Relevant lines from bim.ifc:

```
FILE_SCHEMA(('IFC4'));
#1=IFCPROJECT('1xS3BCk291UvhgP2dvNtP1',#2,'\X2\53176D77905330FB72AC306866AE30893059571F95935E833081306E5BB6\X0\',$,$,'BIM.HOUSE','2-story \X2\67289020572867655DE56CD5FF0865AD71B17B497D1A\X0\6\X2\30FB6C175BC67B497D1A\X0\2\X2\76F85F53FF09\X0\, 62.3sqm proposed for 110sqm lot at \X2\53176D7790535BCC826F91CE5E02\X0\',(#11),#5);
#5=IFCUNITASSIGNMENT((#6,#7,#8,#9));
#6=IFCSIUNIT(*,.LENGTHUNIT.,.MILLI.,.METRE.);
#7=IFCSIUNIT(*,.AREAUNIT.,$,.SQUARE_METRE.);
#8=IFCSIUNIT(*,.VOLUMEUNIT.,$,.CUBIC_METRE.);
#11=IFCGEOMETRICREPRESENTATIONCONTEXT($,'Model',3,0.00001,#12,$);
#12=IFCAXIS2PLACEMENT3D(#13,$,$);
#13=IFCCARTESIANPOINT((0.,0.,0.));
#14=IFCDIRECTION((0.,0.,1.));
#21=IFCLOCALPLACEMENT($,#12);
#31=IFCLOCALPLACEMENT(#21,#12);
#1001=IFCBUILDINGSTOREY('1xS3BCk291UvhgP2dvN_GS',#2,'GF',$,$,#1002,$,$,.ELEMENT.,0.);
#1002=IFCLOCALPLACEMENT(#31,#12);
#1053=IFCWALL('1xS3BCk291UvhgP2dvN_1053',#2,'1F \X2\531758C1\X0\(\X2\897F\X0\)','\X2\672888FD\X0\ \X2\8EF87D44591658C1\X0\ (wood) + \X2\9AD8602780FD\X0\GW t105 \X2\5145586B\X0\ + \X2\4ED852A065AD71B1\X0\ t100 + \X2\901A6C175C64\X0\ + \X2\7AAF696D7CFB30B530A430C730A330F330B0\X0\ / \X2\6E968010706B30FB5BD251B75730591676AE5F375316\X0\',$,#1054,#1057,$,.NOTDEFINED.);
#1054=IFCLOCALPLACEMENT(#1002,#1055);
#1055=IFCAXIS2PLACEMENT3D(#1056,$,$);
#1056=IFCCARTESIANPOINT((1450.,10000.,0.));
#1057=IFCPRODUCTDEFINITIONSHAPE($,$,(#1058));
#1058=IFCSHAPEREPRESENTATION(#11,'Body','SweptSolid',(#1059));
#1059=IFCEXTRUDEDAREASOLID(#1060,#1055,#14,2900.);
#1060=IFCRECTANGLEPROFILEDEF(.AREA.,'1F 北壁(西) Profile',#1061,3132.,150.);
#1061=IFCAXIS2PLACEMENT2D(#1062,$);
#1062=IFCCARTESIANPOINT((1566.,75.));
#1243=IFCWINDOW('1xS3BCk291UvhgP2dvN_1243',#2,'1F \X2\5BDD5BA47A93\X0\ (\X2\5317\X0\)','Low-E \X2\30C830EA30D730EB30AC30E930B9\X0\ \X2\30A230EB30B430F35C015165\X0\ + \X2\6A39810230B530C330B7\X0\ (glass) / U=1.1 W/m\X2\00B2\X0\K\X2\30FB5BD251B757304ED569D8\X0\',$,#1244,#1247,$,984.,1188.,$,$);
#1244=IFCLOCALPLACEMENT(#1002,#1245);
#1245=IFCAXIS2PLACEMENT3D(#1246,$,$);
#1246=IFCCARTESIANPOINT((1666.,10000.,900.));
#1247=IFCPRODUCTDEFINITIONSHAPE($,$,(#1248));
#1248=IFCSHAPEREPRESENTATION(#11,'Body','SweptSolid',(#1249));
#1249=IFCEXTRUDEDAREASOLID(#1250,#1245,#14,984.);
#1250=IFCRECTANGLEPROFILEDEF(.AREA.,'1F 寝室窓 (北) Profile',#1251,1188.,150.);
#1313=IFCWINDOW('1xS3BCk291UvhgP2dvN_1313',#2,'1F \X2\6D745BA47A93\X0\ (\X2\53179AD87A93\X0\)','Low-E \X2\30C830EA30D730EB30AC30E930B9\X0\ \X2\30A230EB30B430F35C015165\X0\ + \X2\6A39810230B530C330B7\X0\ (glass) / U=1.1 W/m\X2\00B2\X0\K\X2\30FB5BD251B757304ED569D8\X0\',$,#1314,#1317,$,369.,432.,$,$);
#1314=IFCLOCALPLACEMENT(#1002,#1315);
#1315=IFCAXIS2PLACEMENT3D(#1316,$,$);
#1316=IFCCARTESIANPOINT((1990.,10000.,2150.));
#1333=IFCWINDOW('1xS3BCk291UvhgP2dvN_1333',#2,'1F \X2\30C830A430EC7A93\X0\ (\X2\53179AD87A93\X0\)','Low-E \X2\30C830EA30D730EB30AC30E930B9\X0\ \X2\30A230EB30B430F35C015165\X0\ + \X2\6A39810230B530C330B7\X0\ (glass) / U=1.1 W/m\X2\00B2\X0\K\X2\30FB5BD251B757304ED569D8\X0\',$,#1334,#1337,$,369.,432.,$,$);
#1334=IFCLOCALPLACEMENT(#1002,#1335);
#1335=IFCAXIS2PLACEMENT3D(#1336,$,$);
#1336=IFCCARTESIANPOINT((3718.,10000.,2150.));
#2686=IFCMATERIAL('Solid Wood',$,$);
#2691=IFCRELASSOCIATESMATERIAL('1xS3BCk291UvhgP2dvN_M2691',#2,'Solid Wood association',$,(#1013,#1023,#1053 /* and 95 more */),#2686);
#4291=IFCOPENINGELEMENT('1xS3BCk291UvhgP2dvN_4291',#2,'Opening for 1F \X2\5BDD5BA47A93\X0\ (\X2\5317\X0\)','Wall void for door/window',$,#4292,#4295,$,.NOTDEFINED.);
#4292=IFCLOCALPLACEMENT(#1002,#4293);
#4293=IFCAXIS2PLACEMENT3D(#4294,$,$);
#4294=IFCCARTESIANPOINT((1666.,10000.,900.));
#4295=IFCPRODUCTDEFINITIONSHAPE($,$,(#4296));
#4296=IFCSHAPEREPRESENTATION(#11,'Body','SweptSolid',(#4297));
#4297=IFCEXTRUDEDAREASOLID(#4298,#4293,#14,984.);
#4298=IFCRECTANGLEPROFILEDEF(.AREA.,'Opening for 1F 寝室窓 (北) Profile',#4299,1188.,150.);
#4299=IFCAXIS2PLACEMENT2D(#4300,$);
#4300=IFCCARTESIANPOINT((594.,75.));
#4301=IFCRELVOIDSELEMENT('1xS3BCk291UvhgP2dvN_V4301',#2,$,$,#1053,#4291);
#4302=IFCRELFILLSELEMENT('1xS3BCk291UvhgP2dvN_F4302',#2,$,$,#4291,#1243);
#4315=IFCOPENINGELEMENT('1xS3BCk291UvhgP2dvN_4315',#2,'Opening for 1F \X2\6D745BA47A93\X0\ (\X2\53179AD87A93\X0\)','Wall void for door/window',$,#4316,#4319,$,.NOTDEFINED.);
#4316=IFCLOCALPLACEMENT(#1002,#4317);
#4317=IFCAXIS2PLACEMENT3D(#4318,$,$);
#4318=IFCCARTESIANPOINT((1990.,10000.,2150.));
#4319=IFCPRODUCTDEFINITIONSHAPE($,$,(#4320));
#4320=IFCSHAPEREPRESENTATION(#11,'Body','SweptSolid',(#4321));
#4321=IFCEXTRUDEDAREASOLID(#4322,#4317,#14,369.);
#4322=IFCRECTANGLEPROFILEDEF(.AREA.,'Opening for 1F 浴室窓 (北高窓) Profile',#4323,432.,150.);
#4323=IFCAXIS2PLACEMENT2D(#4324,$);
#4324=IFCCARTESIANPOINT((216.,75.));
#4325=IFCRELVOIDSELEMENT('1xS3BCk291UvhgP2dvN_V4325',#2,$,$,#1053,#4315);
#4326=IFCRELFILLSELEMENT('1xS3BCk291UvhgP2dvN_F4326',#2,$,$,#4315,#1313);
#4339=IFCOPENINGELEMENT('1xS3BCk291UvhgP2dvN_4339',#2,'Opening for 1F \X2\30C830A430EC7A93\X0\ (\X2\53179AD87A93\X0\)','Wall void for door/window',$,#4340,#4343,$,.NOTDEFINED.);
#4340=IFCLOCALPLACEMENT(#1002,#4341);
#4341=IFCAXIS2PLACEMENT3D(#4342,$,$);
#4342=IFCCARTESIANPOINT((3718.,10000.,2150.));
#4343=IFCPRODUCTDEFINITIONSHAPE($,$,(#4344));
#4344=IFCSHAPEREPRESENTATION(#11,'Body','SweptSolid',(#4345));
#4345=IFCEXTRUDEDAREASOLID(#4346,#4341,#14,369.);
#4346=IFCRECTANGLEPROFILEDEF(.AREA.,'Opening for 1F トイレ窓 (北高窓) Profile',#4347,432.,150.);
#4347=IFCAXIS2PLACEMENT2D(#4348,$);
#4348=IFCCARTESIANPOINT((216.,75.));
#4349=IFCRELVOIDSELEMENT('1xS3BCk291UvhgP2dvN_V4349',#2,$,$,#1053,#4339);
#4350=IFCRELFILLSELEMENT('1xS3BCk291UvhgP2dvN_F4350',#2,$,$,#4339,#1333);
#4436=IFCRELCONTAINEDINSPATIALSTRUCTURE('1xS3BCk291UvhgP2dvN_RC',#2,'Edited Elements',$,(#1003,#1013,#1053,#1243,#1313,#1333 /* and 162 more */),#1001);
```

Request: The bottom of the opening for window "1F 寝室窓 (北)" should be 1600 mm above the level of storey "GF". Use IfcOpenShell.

```python
import numpy as np
import ifcopenshell
import ifcopenshell.api.geometry
import ifcopenshell.geom
import ifcopenshell.util.element
import ifcopenshell.util.placement
import ifcopenshell.util.shape
import ifcopenshell.util.unit

model = ifcopenshell.open("bim.ifc")
unit_scale = ifcopenshell.util.unit.calculate_unit_scale(model)

window = model.by_guid("1xS3BCk291UvhgP2dvN_1243")
opening = window.FillsVoids[0].RelatingOpeningElement
storey = ifcopenshell.util.element.get_container(window, ifc_class="IfcBuildingStorey")
level = ifcopenshell.util.placement.get_local_placement(storey.ObjectPlacement)[2, 3]

# The opening's origin need not be at the sill, so measure its lowest point.
shape = ifcopenshell.geom.create_shape(ifcopenshell.geom.settings(), opening)
bottom = ifcopenshell.util.shape.get_shape_bottom_elevation(shape, shape.geometry) / unit_scale
dz = level + 1.6 / unit_scale - bottom

shift = np.array([0.0, 0.0, dz])
# The window is not placed relative to its opening, so move both.
for product in (opening, window):
    matrix = ifcopenshell.util.placement.get_local_placement(product.ObjectPlacement)
    matrix[:3, 3] += shift
    ifcopenshell.api.geometry.edit_object_placement(model, product=product, matrix=matrix, is_si=False)

print(f"moved by {dz * unit_scale:+.3f} m")

model.write("bim_edited.ifc")
```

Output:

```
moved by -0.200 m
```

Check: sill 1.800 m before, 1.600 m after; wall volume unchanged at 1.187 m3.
